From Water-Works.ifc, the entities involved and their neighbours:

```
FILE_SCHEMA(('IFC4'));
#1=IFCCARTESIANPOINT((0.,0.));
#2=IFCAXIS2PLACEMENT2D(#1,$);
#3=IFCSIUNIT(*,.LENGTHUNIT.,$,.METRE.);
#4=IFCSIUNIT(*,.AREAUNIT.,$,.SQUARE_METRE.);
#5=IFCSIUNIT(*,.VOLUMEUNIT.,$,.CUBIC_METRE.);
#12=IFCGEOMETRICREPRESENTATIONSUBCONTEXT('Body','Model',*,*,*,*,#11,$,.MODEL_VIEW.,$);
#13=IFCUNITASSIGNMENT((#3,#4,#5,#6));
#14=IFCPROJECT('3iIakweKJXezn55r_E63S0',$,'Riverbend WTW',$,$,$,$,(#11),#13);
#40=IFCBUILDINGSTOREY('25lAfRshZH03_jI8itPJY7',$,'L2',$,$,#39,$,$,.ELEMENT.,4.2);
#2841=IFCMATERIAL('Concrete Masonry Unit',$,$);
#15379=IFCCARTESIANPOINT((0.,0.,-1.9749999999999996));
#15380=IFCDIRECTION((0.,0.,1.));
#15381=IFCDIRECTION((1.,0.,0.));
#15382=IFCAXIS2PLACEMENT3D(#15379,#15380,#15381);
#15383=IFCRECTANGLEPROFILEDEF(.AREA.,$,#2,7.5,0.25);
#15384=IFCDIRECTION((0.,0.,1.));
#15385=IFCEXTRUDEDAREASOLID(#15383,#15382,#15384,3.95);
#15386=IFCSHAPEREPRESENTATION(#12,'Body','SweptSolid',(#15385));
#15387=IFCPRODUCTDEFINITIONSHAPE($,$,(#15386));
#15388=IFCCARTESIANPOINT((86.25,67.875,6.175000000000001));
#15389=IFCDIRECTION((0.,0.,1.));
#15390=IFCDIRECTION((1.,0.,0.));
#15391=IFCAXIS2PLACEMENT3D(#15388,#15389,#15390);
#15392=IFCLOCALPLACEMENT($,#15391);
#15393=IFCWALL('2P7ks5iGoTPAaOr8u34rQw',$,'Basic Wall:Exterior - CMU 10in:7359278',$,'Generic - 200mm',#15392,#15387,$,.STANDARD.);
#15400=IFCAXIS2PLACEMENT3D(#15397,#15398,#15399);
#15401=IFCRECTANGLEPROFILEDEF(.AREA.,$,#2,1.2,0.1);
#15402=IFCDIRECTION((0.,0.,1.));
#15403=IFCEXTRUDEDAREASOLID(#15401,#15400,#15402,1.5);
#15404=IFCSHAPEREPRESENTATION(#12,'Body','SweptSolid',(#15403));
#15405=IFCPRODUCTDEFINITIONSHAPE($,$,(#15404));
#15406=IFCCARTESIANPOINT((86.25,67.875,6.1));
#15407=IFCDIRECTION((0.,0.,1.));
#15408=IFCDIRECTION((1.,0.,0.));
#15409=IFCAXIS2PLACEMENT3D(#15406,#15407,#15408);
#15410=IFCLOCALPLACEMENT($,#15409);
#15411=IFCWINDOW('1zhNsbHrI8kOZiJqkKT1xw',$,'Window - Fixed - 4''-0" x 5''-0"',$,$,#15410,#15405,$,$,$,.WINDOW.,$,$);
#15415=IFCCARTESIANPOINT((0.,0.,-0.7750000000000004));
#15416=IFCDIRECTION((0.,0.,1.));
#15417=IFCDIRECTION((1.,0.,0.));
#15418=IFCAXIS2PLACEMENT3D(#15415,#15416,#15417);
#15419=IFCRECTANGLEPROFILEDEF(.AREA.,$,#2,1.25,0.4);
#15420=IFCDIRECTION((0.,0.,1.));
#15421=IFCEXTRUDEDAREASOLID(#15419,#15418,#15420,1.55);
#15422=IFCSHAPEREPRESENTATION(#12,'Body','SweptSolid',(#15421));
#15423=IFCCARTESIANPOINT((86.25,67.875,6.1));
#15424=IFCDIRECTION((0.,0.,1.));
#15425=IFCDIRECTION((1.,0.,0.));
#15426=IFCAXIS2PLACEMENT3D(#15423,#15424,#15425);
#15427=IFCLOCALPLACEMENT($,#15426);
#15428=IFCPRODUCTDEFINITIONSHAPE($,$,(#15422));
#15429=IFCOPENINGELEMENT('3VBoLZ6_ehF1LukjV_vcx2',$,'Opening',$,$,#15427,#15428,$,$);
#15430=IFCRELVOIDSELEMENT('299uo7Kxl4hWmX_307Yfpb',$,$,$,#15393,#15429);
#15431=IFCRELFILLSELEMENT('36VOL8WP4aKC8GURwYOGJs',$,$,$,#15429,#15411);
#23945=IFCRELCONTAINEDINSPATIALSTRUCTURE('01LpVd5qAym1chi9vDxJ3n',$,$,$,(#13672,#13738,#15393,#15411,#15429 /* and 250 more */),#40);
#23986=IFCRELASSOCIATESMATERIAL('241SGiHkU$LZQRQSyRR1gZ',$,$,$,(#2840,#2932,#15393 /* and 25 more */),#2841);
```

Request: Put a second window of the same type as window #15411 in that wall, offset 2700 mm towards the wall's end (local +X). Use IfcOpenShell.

```python
import ifcopenshell
import ifcopenshell.api.feature
import ifcopenshell.api.geometry
import ifcopenshell.api.root
import ifcopenshell.geom
import ifcopenshell.util.element
import ifcopenshell.util.placement
import ifcopenshell.util.shape

model = ifcopenshell.open("Water-Works.ifc")
settings = ifcopenshell.geom.settings()


def volume(element):
    """Net volume in cubic metres, openings subtracted."""
    shape = ifcopenshell.geom.create_shape(settings, element)
    return ifcopenshell.util.shape.get_volume(shape.geometry)


window = model.by_guid("1zhNsbHrI8kOZiJqkKT1xw")
opening = window.FillsVoids[0].RelatingOpeningElement
wall = opening.VoidsElements[0].RelatingBuildingElement
before = volume(wall)
shift = ifcopenshell.util.placement.get_local_placement(wall.ObjectPlacement)[:3, 0] * 2.7

# copy_class copies the void relationship, type, container and properties, but no geometry.
new_opening = ifcopenshell.api.root.copy_class(model, product=opening)
new_opening.Representation = ifcopenshell.util.element.copy_deep(
    model, opening.Representation, exclude=["IfcGeometricRepresentationContext", "IfcRepresentationMap"]
)
new_window = ifcopenshell.api.root.copy_class(model, product=window)
new_window.Representation = ifcopenshell.util.element.copy_deep(
    model, window.Representation, exclude=["IfcGeometricRepresentationContext", "IfcRepresentationMap"]
)
ifcopenshell.api.feature.add_filling(model, opening=new_opening, element=new_window)

for old, new in ((opening, new_opening), (window, new_window)):
    matrix = ifcopenshell.util.placement.get_local_placement(old.ObjectPlacement)
    matrix[:3, 3] += shift
    ifcopenshell.api.geometry.edit_object_placement(model, product=new, matrix=matrix, is_si=False)

after = volume(wall)

print(f"wall volume {before:.3f} -> {after:.3f} m3")

model.write("Water-Works_rev.ifc")
```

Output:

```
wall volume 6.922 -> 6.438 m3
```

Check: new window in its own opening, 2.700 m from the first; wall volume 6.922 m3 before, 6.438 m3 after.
